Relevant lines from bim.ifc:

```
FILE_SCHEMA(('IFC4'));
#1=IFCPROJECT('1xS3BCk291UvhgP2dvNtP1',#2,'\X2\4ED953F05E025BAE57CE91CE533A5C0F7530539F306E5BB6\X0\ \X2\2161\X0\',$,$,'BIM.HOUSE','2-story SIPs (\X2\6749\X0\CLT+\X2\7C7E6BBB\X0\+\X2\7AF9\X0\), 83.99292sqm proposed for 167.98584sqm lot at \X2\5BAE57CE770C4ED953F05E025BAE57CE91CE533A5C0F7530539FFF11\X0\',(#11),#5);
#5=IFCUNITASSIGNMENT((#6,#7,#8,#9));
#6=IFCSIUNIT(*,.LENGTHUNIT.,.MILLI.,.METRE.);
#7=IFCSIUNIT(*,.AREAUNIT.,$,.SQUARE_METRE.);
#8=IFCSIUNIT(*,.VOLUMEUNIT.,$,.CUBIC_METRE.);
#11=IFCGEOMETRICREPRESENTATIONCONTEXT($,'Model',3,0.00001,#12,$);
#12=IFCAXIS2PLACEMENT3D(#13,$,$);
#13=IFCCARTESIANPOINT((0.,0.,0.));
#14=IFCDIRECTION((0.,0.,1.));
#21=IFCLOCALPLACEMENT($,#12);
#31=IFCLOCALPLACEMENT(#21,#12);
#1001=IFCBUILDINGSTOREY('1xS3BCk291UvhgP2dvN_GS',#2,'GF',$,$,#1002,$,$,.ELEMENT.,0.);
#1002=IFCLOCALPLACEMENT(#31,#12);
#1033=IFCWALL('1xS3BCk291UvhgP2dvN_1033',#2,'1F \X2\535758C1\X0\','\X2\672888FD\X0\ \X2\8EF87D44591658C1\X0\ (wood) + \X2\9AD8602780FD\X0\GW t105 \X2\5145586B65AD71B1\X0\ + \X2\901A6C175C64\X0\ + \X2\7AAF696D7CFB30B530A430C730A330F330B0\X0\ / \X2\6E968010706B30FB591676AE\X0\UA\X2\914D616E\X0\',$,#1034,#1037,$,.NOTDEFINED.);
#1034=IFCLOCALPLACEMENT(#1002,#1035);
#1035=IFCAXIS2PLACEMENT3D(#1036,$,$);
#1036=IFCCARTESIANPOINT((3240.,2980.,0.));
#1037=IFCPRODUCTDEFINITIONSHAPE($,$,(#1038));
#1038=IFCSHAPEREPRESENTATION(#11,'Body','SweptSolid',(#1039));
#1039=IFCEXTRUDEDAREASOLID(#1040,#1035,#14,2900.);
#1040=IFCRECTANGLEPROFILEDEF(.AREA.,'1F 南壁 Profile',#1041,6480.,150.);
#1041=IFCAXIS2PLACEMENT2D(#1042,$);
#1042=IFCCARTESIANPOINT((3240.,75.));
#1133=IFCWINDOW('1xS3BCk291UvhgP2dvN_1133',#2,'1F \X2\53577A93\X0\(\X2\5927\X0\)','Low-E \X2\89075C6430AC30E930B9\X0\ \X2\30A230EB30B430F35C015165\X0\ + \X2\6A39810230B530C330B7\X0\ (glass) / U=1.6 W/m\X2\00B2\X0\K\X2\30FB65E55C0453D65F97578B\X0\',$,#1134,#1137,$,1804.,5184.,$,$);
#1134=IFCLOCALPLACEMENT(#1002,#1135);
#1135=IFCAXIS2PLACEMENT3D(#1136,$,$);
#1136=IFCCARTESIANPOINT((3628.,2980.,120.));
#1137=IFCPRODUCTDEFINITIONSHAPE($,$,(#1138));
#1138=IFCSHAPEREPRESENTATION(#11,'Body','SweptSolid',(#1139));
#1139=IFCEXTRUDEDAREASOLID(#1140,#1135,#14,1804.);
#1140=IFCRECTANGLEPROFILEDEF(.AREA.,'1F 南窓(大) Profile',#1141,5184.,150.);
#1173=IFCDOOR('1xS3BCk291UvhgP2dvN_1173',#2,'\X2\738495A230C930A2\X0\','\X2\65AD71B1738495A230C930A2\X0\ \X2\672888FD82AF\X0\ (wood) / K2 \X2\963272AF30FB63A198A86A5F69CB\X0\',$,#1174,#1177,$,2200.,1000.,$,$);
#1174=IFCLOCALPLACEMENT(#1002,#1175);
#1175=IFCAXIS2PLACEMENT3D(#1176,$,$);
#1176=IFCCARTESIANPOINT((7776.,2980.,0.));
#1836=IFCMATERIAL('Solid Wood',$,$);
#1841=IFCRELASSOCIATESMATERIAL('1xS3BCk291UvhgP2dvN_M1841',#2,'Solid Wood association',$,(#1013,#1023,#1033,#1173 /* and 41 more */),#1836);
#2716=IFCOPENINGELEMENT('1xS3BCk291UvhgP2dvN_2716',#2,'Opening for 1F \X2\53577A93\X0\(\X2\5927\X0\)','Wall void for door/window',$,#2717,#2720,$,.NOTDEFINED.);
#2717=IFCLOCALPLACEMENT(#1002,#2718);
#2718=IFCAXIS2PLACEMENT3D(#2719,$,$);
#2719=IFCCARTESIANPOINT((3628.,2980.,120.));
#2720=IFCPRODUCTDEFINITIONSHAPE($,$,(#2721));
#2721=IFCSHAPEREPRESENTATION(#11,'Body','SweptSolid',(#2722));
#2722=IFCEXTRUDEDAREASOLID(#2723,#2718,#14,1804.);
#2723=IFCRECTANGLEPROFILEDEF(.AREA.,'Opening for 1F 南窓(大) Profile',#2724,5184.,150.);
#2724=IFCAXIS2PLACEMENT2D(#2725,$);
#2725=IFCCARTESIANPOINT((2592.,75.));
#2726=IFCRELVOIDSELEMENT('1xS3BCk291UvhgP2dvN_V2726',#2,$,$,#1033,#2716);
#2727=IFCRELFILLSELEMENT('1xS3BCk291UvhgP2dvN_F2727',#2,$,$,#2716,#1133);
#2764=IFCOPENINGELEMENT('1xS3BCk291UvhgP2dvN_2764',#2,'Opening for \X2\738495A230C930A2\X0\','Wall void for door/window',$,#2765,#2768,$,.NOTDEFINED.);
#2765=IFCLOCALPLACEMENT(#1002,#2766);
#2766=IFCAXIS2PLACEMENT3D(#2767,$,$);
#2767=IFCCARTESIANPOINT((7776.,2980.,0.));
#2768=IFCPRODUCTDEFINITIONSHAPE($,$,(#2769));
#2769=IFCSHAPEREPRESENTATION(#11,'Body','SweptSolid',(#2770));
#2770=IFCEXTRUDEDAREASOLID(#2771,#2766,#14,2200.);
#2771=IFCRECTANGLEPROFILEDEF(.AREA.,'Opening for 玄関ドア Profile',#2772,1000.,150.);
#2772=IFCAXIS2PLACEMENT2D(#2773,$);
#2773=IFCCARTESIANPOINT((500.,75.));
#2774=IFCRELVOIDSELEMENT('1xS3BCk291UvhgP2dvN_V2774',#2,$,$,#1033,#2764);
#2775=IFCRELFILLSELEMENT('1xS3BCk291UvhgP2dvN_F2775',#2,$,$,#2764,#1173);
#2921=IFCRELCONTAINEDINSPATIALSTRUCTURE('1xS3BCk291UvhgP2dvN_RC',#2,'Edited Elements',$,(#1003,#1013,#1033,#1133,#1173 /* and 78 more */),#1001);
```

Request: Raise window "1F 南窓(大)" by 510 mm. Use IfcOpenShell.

```python
import numpy as np
import ifcopenshell
import ifcopenshell.api.geometry
import ifcopenshell.util.placement
import ifcopenshell.util.unit

model = ifcopenshell.open("bim.ifc")
unit_scale = ifcopenshell.util.unit.calculate_unit_scale(model)

window = model.by_guid("1xS3BCk291UvhgP2dvN_1133")
opening = window.FillsVoids[0].RelatingOpeningElement
dz = 0.51 / unit_scale

shift = np.array([0.0, 0.0, dz])
# The window is not placed relative to its opening, so move both.
for product in (opening, window):
    matrix = ifcopenshell.util.placement.get_local_placement(product.ObjectPlacement)
    matrix[:3, 3] += shift
    ifcopenshell.api.geometry.edit_object_placement(model, product=product, matrix=matrix, is_si=False)

print(f"moved by {dz * unit_scale:+.3f} m")

model.write("bim-out.ifc")
```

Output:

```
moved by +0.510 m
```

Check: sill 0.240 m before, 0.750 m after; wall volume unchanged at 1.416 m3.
